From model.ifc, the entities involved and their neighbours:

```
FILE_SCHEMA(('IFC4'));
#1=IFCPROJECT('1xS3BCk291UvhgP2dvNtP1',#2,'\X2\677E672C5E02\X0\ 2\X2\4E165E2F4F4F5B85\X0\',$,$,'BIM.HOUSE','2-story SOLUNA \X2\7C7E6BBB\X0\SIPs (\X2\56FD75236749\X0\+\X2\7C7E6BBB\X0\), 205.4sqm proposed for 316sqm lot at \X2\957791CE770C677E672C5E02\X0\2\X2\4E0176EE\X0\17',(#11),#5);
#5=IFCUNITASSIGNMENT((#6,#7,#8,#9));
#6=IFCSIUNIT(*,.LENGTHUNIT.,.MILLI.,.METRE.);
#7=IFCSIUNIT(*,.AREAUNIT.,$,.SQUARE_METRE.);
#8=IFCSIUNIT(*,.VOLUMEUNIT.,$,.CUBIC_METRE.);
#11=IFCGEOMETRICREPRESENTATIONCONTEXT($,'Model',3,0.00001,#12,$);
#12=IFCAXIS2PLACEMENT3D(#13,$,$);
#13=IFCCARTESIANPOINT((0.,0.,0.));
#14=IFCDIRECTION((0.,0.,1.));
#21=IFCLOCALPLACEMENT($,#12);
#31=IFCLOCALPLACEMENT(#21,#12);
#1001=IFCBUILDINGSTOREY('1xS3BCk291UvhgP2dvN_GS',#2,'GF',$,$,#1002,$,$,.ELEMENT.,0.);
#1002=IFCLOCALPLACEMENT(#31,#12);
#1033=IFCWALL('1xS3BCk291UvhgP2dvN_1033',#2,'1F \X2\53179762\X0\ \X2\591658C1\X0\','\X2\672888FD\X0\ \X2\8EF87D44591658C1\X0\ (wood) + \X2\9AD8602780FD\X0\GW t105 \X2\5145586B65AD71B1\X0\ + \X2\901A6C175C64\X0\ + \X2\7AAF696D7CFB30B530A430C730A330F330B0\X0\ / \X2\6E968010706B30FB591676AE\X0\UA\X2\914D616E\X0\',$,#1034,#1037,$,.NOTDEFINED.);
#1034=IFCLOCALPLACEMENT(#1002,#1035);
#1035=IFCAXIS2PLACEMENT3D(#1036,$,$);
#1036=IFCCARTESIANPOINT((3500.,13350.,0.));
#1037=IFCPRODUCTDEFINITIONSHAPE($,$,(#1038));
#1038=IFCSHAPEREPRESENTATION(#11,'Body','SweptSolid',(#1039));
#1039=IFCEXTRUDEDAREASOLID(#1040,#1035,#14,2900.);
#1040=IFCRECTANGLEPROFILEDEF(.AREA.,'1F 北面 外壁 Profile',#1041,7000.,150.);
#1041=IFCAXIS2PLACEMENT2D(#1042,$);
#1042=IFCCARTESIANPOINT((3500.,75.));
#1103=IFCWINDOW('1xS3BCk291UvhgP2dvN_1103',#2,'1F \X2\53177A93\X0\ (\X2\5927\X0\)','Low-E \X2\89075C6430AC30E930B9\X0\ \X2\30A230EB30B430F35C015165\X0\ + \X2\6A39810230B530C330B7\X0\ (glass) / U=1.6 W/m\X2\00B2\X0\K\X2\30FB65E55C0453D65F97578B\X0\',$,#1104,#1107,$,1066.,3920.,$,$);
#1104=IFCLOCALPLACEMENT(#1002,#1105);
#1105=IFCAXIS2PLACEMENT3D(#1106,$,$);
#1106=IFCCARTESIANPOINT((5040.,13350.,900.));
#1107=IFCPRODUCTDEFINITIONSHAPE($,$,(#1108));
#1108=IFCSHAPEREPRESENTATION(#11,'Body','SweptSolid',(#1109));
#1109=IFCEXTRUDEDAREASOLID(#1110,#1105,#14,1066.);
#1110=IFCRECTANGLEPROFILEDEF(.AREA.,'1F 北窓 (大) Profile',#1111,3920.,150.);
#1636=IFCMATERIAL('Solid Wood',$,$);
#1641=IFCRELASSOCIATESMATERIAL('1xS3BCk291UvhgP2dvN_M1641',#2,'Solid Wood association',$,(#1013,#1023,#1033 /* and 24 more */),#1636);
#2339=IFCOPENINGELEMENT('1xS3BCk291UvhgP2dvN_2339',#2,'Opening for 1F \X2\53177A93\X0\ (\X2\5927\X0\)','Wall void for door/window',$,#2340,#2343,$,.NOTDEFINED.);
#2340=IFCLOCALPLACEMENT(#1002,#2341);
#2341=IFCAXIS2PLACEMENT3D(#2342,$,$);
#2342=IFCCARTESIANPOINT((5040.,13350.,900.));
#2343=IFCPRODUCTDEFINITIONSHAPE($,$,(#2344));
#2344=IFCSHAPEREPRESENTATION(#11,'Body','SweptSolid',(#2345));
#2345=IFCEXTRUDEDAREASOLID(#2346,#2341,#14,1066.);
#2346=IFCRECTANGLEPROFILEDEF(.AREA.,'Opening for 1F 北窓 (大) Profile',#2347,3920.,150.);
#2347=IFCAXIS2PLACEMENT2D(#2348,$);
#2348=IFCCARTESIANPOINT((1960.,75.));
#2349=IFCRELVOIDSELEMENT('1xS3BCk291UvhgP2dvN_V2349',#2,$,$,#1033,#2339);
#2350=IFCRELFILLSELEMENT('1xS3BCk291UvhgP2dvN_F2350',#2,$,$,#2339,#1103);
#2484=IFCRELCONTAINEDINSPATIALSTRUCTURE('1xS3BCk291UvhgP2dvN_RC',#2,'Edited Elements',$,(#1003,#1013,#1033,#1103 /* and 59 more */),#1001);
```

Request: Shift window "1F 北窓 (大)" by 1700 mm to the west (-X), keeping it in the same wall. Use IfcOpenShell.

```python
import ifcopenshell
import ifcopenshell.api.geometry
import ifcopenshell.util.placement
import ifcopenshell.util.unit

model = ifcopenshell.open("model.ifc")
unit_scale = ifcopenshell.util.unit.calculate_unit_scale(model)

window = model.by_guid("1xS3BCk291UvhgP2dvN_1103")
opening = window.FillsVoids[0].RelatingOpeningElement
wall = opening.VoidsElements[0].RelatingBuildingElement

wall_matrix = ifcopenshell.util.placement.get_local_placement(wall.ObjectPlacement)
shift = wall_matrix[:3, 0] * -1.7 / unit_scale
before = ifcopenshell.util.placement.get_local_placement(window.ObjectPlacement)[:3, 3].copy()

# The window is not placed relative to its opening, so move both.
for product in (opening, window):
    matrix = ifcopenshell.util.placement.get_local_placement(product.ObjectPlacement)
    matrix[:3, 3] += shift
    ifcopenshell.api.geometry.edit_object_placement(model, product=product, matrix=matrix, is_si=False)

after = ifcopenshell.util.placement.get_local_placement(window.ObjectPlacement)[:3, 3]
print("window moved by", (after - before).round(3) + 0.0)

model.write("model-out.ifc")
```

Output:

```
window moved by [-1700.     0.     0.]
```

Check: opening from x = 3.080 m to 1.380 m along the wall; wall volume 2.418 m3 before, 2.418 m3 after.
